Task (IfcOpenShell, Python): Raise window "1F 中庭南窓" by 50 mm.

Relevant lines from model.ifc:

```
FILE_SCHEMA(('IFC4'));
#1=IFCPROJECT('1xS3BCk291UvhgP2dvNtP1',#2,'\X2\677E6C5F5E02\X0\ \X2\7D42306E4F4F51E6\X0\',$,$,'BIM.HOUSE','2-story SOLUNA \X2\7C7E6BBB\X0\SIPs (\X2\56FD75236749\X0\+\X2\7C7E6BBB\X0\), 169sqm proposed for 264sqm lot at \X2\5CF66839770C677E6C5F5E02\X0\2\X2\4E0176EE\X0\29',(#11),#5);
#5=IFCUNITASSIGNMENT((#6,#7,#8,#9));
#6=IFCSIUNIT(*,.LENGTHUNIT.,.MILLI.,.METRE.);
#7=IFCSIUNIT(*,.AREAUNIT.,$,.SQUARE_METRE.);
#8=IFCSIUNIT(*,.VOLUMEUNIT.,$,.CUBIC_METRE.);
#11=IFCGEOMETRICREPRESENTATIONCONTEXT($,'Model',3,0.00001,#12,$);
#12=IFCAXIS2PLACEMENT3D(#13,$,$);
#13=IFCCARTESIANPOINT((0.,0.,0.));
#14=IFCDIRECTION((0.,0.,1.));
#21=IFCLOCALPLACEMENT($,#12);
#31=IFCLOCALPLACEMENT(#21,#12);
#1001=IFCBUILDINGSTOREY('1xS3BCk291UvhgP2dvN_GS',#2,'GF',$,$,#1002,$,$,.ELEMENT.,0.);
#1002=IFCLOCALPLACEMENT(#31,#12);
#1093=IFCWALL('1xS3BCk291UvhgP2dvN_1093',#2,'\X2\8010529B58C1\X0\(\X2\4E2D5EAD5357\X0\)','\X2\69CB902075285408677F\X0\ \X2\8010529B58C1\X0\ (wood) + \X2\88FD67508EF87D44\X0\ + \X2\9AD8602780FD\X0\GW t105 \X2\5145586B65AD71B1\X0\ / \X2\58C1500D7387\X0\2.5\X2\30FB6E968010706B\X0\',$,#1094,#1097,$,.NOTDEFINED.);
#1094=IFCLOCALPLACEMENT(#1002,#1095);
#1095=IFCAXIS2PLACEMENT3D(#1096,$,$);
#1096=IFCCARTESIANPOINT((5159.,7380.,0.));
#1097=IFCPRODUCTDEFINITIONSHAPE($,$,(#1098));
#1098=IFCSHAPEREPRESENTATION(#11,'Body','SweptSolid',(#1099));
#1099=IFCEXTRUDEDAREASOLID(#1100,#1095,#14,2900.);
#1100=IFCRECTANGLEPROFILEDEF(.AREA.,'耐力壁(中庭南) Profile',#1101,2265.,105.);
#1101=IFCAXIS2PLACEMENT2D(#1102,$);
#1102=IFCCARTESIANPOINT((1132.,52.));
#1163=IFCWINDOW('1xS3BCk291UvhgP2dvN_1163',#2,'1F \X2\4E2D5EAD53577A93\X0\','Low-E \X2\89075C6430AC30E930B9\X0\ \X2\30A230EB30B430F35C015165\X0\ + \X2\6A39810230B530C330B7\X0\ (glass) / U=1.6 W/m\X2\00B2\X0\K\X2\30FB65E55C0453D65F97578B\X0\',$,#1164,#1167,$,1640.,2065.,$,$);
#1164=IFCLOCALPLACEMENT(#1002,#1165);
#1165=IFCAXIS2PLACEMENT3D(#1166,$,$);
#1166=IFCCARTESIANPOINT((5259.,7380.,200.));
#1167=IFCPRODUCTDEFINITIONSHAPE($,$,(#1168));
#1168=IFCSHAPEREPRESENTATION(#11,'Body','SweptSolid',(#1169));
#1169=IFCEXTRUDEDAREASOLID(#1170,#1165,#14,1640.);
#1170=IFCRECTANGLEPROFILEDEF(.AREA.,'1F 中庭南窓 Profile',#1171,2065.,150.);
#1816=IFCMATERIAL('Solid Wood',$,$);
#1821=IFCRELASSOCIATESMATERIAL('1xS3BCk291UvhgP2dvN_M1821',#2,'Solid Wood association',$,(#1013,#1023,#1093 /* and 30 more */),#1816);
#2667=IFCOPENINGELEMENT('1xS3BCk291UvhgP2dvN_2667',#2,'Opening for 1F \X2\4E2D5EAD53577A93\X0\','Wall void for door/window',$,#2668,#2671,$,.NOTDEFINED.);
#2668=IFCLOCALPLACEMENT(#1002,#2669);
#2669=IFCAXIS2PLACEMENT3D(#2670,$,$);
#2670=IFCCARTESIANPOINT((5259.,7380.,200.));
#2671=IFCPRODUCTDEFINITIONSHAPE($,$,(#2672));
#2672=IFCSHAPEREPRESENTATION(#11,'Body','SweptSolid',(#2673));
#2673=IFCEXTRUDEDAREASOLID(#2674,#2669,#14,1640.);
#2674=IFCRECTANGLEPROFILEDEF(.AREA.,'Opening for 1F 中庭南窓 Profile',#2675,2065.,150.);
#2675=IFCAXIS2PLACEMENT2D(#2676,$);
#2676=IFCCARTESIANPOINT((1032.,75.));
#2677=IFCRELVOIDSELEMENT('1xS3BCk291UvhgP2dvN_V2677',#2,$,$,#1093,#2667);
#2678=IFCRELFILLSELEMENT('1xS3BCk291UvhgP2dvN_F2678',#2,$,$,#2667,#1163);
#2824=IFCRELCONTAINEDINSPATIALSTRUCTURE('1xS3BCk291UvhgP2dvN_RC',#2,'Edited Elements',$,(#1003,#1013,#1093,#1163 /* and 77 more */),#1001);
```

```python
import numpy as np
import ifcopenshell
import ifcopenshell.api.geometry
import ifcopenshell.util.placement
import ifcopenshell.util.unit

model = ifcopenshell.open("model.ifc")
unit_scale = ifcopenshell.util.unit.calculate_unit_scale(model)

window = model.by_guid("1xS3BCk291UvhgP2dvN_1163")
opening = window.FillsVoids[0].RelatingOpeningElement
dz = 0.05 / unit_scale

shift = np.array([0.0, 0.0, dz])
# The window is not placed relative to its opening, so move both.
for product in (opening, window):
    matrix = ifcopenshell.util.placement.get_local_placement(product.ObjectPlacement)
    matrix[:3, 3] += shift
    ifcopenshell.api.geometry.edit_object_placement(model, product=product, matrix=matrix, is_si=False)

print(f"moved by {dz * unit_scale:+.3f} m")

model.write("model-out.ifc")
```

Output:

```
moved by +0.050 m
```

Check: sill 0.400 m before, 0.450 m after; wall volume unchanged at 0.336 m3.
